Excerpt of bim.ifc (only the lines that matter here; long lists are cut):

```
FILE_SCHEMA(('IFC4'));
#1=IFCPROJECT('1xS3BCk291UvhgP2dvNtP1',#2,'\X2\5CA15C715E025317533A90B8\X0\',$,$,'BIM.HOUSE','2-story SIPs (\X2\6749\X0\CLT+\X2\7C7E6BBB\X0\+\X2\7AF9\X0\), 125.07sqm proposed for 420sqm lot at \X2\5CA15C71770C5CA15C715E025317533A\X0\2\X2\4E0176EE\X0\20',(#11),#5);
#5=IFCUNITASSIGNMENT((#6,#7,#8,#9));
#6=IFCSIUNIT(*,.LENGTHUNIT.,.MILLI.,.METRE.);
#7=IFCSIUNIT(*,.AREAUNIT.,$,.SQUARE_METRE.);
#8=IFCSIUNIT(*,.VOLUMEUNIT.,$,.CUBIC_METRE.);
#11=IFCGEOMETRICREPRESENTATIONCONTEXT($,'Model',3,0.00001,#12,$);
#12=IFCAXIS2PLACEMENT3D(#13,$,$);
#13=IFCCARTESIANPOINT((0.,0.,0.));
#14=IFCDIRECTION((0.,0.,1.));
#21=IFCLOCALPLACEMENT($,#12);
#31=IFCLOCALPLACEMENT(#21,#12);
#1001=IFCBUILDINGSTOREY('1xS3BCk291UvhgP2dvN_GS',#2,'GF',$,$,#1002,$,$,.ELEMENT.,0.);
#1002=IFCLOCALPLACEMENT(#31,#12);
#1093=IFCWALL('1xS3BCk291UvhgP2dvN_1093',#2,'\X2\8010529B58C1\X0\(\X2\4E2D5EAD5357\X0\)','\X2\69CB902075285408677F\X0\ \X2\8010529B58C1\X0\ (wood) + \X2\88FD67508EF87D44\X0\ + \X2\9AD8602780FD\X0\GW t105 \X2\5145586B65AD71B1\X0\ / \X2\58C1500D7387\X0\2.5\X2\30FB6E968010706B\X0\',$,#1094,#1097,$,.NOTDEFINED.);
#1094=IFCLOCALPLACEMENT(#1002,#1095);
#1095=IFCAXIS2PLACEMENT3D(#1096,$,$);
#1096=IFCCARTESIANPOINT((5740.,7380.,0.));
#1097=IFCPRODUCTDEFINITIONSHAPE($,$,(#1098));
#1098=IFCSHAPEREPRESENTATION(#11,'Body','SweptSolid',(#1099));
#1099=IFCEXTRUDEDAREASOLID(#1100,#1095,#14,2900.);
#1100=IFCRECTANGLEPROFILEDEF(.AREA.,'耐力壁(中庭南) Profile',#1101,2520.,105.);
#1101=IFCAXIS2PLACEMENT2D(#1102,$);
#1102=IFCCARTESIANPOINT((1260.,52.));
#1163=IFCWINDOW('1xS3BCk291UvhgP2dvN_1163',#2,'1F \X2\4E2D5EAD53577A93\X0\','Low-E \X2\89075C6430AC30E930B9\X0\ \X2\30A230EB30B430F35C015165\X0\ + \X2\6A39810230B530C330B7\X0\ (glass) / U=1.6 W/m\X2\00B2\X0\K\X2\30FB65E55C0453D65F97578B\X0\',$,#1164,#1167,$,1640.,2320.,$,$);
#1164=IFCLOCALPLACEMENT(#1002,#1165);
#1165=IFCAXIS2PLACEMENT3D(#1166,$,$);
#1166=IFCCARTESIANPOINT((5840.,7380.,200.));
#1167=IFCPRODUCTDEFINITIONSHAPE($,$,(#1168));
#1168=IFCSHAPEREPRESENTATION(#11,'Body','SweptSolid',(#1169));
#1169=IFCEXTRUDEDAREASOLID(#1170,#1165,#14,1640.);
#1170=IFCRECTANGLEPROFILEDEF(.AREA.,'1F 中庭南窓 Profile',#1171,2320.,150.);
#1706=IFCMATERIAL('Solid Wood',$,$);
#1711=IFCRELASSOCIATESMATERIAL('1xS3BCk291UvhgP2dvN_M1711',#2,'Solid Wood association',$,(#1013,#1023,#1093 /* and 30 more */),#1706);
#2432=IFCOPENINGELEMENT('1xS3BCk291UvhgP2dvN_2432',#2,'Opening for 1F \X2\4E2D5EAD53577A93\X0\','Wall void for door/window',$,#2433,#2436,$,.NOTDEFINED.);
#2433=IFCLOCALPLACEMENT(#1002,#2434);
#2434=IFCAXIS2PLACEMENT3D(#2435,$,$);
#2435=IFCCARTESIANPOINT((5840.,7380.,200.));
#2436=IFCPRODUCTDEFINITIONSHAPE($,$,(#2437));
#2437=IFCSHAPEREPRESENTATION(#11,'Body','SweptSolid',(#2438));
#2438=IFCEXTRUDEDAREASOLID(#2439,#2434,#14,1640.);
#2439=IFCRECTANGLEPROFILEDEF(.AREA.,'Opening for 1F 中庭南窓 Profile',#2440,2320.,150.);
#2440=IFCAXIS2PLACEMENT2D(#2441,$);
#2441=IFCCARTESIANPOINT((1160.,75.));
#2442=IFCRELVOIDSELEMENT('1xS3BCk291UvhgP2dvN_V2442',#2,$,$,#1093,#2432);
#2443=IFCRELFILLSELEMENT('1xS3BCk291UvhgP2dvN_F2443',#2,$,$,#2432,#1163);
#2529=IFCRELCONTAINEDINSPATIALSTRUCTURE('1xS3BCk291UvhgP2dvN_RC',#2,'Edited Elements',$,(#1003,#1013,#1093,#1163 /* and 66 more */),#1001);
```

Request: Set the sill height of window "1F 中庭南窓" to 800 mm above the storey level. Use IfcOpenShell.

```python
import numpy as np
import ifcopenshell
import ifcopenshell.api.geometry
import ifcopenshell.geom
import ifcopenshell.util.element
import ifcopenshell.util.placement
import ifcopenshell.util.shape
import ifcopenshell.util.unit

model = ifcopenshell.open("bim.ifc")
unit_scale = ifcopenshell.util.unit.calculate_unit_scale(model)

window = model.by_guid("1xS3BCk291UvhgP2dvN_1163")
opening = window.FillsVoids[0].RelatingOpeningElement
storey = ifcopenshell.util.element.get_container(window, ifc_class="IfcBuildingStorey")
level = ifcopenshell.util.placement.get_local_placement(storey.ObjectPlacement)[2, 3]

# The opening's origin need not be at the sill, so measure its lowest point.
shape = ifcopenshell.geom.create_shape(ifcopenshell.geom.settings(), opening)
bottom = ifcopenshell.util.shape.get_shape_bottom_elevation(shape, shape.geometry) / unit_scale
dz = level + 0.8 / unit_scale - bottom

shift = np.array([0.0, 0.0, dz])
# The window is not placed relative to its opening, so move both.
for product in (opening, window):
    matrix = ifcopenshell.util.placement.get_local_placement(product.ObjectPlacement)
    matrix[:3, 3] += shift
    ifcopenshell.api.geometry.edit_object_placement(model, product=product, matrix=matrix, is_si=False)

print(f"moved by {dz * unit_scale:+.3f} m")

model.write("bim_v2.ifc")
```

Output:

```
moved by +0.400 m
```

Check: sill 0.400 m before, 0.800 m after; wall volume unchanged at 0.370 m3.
